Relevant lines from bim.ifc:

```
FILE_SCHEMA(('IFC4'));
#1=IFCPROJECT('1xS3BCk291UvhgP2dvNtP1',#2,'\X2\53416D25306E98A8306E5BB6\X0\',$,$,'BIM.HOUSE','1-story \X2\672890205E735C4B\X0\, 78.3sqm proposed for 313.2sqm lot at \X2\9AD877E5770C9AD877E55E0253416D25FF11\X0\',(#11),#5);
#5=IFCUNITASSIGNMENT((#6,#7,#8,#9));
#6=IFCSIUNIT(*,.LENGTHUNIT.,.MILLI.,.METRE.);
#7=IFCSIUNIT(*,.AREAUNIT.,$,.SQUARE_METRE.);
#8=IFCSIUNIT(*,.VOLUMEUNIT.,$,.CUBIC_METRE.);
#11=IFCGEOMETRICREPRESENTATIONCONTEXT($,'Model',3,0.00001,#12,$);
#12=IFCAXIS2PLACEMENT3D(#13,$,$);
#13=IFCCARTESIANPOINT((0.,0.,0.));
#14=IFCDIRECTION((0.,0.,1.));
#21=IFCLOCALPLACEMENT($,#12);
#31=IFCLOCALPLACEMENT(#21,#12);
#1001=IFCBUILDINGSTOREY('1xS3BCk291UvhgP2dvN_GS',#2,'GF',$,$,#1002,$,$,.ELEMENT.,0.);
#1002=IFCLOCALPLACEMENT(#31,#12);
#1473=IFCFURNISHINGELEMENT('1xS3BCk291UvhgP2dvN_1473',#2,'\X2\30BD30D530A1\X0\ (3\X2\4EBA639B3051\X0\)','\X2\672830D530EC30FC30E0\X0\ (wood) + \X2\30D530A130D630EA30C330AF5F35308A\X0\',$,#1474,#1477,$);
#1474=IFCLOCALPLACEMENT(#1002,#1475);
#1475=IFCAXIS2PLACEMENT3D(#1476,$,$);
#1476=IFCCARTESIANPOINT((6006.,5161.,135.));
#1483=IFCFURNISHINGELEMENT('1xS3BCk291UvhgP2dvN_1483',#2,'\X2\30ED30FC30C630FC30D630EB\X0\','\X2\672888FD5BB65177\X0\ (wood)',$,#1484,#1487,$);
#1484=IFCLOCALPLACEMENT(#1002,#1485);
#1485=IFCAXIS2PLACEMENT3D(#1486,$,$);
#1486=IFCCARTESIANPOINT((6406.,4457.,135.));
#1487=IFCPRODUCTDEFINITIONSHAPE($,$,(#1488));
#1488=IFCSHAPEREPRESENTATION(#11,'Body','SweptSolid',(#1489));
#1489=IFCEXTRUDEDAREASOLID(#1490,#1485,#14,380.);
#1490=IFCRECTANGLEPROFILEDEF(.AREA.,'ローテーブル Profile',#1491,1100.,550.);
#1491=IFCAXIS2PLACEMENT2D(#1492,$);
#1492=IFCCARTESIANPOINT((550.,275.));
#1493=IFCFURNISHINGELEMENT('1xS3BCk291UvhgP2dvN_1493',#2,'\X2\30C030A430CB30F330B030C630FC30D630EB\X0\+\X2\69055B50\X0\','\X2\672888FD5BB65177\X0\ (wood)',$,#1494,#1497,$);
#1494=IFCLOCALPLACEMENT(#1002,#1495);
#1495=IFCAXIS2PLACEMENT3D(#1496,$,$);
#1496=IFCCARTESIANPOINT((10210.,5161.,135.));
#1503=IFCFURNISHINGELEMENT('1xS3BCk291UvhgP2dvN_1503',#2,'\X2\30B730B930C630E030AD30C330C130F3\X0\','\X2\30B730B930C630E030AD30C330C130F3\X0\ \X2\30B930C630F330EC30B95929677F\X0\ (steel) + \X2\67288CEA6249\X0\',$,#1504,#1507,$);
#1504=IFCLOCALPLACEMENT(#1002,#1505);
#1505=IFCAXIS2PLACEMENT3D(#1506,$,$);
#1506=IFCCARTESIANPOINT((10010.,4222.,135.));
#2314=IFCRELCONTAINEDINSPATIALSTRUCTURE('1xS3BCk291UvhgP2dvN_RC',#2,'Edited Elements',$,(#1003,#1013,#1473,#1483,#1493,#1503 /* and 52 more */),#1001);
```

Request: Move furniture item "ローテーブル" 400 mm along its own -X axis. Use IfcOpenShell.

```python
import ifcopenshell
import ifcopenshell.api.geometry
import ifcopenshell.util.placement
import ifcopenshell.util.unit

model = ifcopenshell.open("bim.ifc")
unit_scale = ifcopenshell.util.unit.calculate_unit_scale(model)

item = model.by_id(1483)
matrix = ifcopenshell.util.placement.get_local_placement(item.ObjectPlacement)
matrix[:3, 3] -= matrix[:3, 0] * 0.4 / unit_scale
ifcopenshell.api.geometry.edit_object_placement(model, product=item, matrix=matrix, is_si=False)

print(ifcopenshell.util.placement.get_local_placement(item.ObjectPlacement).round(3) + 0.0)

model.write("bim_rev.ifc")
```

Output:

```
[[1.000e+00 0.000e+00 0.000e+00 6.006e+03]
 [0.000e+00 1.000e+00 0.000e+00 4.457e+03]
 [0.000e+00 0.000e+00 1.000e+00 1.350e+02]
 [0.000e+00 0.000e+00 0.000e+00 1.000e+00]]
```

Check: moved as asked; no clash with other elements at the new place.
